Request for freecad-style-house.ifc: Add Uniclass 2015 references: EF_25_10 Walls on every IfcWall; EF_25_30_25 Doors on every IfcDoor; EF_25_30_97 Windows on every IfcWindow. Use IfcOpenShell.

First a look at what the model holds.

```python
import ifcopenshell

model = ifcopenshell.open("freecad-style-house.ifc")
print(model.schema)
print("classifications:", [c.Name for c in model.by_type("IfcClassification")])
for ifc_class in ("IfcDoor", "IfcRoof", "IfcStair", "IfcWall", "IfcWindow"):
    print(ifc_class, len(model.by_type(ifc_class)))
```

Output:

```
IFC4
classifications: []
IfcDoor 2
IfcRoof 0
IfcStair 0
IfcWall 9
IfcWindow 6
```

```python
import ifcopenshell
import ifcopenshell.api.classification

model = ifcopenshell.open("freecad-style-house.ifc")

system = ifcopenshell.api.classification.add_classification(model, classification="Uniclass 2015")

codes = {
    "IfcWall": ("EF_25_10", "Walls"),
    "IfcDoor": ("EF_25_30_25", "Doors"),
    "IfcWindow": ("EF_25_30_97", "Windows"),
}
for ifc_class, (code, name) in codes.items():
    products = model.by_type(ifc_class)
    ifcopenshell.api.classification.add_reference(
        model, products=products, classification=system, identification=code, name=name
    )
    print(code, len(products))

model.write("freecad-style-house_updated.ifc")
```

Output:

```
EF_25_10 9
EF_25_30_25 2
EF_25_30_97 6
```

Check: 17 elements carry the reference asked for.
